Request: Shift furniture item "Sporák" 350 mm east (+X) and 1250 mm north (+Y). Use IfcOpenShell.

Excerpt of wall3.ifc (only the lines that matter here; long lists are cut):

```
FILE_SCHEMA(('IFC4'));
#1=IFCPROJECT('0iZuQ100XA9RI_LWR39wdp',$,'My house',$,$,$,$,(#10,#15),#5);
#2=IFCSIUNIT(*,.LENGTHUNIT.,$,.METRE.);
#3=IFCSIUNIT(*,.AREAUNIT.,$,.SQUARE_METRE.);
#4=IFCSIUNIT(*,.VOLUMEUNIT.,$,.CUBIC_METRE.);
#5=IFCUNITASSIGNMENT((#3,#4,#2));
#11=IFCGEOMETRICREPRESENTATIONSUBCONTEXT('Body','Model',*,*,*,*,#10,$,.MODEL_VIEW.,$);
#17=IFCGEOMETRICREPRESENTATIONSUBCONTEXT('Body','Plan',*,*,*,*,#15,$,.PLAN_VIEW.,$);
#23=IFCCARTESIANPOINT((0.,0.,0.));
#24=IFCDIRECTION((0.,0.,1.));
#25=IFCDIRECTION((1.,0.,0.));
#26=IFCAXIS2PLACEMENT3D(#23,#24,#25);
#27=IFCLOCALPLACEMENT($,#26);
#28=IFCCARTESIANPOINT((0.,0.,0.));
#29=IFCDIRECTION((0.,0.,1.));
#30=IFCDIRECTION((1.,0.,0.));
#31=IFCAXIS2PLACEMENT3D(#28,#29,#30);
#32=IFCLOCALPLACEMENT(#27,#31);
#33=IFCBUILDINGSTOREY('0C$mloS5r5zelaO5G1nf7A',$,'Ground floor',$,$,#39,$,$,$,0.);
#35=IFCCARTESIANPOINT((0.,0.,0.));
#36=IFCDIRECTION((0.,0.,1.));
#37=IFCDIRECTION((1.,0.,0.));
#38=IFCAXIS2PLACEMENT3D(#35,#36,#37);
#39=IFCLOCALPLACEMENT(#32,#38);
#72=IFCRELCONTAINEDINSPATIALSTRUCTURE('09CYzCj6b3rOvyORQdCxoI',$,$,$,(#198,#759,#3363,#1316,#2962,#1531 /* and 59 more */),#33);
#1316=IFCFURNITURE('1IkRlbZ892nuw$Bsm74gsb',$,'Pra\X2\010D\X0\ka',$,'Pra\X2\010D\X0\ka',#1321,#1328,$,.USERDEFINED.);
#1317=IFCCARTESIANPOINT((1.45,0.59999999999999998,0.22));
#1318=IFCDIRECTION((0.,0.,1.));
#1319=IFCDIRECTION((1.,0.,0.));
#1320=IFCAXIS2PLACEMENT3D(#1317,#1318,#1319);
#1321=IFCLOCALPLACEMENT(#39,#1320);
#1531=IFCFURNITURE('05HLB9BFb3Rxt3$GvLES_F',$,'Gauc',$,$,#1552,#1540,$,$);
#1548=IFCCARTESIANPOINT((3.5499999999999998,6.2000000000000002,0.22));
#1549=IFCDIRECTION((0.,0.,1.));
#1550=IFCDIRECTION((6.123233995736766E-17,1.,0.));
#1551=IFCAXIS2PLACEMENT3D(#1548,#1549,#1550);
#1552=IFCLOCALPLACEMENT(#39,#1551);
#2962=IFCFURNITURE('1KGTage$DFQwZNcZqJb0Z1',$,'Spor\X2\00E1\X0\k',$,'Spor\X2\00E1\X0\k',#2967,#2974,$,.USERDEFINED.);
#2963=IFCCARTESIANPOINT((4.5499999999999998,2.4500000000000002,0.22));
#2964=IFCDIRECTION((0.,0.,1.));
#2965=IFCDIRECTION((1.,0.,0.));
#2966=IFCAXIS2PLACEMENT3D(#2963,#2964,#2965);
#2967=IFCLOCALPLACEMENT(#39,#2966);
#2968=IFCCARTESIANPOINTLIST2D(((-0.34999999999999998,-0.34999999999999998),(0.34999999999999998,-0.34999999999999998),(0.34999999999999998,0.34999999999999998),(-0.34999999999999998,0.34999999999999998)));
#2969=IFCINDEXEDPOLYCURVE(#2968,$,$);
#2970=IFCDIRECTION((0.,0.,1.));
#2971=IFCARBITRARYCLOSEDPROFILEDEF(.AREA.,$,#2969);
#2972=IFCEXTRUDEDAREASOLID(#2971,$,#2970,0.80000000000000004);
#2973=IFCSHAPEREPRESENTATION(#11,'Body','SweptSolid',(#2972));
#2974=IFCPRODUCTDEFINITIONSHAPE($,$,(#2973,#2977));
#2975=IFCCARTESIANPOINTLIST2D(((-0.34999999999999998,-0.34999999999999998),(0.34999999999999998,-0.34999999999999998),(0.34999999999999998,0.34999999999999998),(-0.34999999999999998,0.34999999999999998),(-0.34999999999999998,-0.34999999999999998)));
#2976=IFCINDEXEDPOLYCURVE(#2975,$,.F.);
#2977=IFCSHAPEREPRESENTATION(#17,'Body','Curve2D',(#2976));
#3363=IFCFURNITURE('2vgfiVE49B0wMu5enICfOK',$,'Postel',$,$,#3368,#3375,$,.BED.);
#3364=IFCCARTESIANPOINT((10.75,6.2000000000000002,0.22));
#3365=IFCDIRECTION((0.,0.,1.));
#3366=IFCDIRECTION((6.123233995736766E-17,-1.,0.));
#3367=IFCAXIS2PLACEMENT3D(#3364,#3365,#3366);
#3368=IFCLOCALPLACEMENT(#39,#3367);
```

```python
import ifcopenshell
import ifcopenshell.api.geometry
import ifcopenshell.util.placement

model = ifcopenshell.open("wall3.ifc")

item = model.by_guid("1KGTage$DFQwZNcZqJb0Z1")
matrix = ifcopenshell.util.placement.get_local_placement(item.ObjectPlacement)
matrix[0, 3] += 0.35
matrix[1, 3] += 1.25
ifcopenshell.api.geometry.edit_object_placement(model, product=item, matrix=matrix, is_si=False)

print(ifcopenshell.util.placement.get_local_placement(item.ObjectPlacement).round(3) + 0.0)

model.write("wall3_v2.ifc")
```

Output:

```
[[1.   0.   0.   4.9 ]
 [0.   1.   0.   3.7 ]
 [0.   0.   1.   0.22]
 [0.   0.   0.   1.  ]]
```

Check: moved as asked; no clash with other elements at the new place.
